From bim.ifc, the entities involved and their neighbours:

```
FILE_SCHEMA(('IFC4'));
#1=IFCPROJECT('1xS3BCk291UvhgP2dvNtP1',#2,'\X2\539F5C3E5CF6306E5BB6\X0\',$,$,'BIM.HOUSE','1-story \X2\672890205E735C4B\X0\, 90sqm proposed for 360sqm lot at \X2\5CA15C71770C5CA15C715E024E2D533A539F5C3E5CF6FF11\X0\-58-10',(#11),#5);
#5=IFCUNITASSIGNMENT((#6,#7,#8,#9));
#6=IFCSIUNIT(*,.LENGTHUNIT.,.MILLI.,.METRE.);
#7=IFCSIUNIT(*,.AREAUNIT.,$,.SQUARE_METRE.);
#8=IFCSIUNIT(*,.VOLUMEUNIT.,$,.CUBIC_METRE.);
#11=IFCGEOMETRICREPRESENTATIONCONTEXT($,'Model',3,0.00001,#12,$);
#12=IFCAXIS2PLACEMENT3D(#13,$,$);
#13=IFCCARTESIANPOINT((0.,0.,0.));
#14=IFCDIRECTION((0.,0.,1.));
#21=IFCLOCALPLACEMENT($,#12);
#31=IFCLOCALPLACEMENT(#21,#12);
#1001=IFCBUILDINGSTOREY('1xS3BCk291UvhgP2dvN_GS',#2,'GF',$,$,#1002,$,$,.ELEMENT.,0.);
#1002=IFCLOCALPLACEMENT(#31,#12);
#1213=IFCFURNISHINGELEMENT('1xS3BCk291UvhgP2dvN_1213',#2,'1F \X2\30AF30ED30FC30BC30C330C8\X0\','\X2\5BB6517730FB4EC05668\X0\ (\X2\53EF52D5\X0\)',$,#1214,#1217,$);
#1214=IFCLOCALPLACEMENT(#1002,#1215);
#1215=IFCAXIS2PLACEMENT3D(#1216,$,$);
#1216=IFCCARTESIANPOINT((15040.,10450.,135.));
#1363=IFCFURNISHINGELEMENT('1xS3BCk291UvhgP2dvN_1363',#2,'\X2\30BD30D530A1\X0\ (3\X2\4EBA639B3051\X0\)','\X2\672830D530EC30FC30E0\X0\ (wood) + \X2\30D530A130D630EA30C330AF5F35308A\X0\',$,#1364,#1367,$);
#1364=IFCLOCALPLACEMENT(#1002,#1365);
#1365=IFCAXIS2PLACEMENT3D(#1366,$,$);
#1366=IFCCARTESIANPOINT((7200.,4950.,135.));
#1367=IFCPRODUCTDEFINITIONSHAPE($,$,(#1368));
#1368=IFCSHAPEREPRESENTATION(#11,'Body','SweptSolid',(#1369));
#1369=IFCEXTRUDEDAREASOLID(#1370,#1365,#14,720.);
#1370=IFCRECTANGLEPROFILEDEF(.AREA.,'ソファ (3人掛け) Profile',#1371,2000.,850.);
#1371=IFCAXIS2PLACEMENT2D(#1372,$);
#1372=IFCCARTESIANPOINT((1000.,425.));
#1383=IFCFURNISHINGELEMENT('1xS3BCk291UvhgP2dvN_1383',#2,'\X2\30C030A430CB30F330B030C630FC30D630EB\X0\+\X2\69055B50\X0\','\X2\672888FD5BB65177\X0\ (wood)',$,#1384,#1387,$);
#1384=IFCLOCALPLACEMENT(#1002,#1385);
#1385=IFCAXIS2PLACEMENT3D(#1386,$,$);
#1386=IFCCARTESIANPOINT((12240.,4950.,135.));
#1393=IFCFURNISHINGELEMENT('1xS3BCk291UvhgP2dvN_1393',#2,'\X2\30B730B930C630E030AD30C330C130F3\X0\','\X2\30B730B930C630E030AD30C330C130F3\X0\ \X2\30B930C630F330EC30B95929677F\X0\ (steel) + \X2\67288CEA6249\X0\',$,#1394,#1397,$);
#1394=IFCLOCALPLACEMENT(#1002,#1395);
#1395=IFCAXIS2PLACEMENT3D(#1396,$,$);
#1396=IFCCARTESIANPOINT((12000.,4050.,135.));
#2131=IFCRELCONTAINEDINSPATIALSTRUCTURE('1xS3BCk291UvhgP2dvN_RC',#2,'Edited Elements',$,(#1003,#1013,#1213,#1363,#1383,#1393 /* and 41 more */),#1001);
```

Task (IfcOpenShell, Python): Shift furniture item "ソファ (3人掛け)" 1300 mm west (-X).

```python
import ifcopenshell
import ifcopenshell.api.geometry
import ifcopenshell.util.placement

model = ifcopenshell.open("bim.ifc")

item = model.by_id(1363)
matrix = ifcopenshell.util.placement.get_local_placement(item.ObjectPlacement)
matrix[0, 3] -= 1300.0
ifcopenshell.api.geometry.edit_object_placement(model, product=item, matrix=matrix, is_si=False)

print(ifcopenshell.util.placement.get_local_placement(item.ObjectPlacement).round(3) + 0.0)

model.write("bim_updated.ifc")
```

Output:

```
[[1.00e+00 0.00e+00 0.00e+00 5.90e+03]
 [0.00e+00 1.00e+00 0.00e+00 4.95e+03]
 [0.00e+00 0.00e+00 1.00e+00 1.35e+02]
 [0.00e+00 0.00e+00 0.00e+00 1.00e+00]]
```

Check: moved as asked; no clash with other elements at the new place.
